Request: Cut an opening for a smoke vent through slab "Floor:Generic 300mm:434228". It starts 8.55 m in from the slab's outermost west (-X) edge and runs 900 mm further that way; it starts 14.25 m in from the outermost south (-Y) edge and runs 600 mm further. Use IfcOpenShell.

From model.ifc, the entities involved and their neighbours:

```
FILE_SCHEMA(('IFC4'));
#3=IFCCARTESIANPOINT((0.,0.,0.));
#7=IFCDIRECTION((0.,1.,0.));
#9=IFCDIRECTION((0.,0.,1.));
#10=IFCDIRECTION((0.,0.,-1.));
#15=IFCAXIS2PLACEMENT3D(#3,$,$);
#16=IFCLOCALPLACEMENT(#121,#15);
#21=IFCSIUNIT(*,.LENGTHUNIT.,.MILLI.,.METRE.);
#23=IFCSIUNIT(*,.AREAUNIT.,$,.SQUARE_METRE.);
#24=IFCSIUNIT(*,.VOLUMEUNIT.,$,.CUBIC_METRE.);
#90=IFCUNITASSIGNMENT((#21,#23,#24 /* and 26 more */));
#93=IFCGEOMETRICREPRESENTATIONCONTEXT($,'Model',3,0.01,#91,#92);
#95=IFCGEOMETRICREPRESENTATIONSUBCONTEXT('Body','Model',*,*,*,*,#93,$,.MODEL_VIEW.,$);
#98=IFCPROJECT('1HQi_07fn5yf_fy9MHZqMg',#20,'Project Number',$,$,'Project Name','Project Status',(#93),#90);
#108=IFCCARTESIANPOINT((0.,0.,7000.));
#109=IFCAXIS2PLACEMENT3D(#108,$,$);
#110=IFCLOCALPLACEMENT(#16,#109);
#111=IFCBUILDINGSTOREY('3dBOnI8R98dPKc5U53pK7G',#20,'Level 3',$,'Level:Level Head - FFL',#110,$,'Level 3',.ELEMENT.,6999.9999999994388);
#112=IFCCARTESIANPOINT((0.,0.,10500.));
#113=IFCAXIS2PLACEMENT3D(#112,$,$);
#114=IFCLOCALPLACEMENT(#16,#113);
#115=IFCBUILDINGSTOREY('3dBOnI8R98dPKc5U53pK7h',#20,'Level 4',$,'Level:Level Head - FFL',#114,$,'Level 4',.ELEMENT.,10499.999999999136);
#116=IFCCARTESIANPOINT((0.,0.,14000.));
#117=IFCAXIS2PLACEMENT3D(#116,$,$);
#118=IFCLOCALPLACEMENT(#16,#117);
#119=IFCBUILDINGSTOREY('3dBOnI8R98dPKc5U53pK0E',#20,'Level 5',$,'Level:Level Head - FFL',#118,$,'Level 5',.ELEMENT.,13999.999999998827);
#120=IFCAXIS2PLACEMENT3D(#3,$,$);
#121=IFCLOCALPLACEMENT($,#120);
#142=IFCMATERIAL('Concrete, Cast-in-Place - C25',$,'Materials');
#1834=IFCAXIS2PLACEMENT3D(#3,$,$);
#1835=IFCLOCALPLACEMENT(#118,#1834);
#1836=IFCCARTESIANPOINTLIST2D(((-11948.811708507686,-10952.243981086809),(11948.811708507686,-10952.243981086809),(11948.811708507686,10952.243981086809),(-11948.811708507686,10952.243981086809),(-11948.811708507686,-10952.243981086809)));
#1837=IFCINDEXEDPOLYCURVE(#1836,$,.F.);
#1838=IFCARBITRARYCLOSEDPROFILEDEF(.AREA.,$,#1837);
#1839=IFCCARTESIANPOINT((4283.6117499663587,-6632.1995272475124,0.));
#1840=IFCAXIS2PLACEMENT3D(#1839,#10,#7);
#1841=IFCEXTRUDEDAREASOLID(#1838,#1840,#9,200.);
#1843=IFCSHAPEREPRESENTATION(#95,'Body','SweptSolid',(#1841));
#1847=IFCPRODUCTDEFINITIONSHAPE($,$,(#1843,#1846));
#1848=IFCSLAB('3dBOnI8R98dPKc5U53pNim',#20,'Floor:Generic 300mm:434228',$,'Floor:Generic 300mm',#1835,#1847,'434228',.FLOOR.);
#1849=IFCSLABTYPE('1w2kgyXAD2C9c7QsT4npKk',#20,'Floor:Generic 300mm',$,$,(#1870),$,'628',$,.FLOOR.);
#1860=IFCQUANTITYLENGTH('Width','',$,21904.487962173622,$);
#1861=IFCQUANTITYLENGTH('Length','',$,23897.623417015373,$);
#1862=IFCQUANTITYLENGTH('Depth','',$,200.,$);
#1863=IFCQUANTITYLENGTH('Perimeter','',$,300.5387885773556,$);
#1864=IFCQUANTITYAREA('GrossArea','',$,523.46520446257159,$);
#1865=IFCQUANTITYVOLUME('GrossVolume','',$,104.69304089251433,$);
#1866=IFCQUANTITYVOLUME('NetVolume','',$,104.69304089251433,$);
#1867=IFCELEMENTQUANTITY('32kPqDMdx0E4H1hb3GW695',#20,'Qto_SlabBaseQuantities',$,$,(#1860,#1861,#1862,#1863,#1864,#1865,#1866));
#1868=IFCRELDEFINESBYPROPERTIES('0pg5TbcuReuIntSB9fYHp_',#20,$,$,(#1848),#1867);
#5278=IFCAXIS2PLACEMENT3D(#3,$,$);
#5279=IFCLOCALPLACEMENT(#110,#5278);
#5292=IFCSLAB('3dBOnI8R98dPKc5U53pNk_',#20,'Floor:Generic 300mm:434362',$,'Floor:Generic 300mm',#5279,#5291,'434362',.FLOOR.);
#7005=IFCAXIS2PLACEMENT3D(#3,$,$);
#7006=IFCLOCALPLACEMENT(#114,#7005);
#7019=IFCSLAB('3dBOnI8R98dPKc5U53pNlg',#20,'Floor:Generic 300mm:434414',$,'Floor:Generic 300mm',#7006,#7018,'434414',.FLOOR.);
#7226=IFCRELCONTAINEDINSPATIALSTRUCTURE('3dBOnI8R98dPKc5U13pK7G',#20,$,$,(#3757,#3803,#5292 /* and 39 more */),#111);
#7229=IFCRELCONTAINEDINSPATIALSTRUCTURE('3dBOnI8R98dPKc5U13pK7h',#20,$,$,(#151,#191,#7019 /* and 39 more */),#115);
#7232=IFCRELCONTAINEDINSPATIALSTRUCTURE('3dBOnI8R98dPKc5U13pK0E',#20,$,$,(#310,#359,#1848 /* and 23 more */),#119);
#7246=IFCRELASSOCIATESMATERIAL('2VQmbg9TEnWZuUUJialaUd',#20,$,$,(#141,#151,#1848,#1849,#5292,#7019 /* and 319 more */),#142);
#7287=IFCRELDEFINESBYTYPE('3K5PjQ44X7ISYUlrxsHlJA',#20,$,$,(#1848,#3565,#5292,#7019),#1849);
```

```python
import numpy as np
import ifcopenshell
import ifcopenshell.api.feature
import ifcopenshell.api.geometry
import ifcopenshell.api.pset
import ifcopenshell.api.root
import ifcopenshell.geom
import ifcopenshell.util.element
import ifcopenshell.util.placement
import ifcopenshell.util.representation
import ifcopenshell.util.shape
import ifcopenshell.util.unit

model = ifcopenshell.open("model.ifc")
unit_scale = ifcopenshell.util.unit.calculate_unit_scale(model)
volume_scale = ifcopenshell.util.unit.calculate_unit_scale(model, "VOLUMEUNIT")
settings = ifcopenshell.geom.settings()


def volume(element):
    """Net volume in cubic metres, openings subtracted."""
    shape = ifcopenshell.geom.create_shape(settings, element)
    return ifcopenshell.util.shape.get_volume(shape.geometry)


slab = model.by_guid("3dBOnI8R98dPKc5U53pNim")
before = volume(slab)

# Extent in the slab's own axes, in metres. The edges named are its -X and -Y sides.
slab_shape = ifcopenshell.geom.create_shape(settings, slab)
vertices = ifcopenshell.util.shape.get_vertices(slab_shape.geometry)
x_min, y_min, bottom = vertices.min(axis=0)
top = vertices[:, 2].max()

opening = ifcopenshell.api.root.create_entity(model, ifc_class="IfcOpeningElement", name="Smoke vent opening", predefined_type="OPENING")
context = ifcopenshell.util.representation.get_context(model, "Model", "Body", "MODEL_VIEW")
width, depth = 0.9, 0.6
outline = [(0.0, 0.0), (width, 0.0), (width, depth), (0.0, depth), (0.0, 0.0)]
# Overshoot both faces by 50 mm so the cut is clean.
shape = ifcopenshell.api.geometry.add_slab_representation(
    model, context=context, depth=top - bottom + 0.1, polyline=outline
)
ifcopenshell.api.geometry.assign_representation(model, product=opening, representation=shape)

matrix = ifcopenshell.util.placement.get_local_placement(slab.ObjectPlacement)
matrix[:, 3] = matrix @ np.append(np.array([x_min + 8.55, y_min + 14.25, bottom - 0.05]) / unit_scale, 1.0)
ifcopenshell.api.geometry.edit_object_placement(model, product=opening, matrix=matrix, is_si=False)
ifcopenshell.api.feature.add_feature(model, feature=opening, element=slab)

after = volume(slab)

# Update the slab's stored quantities.
qto = model.by_id(ifcopenshell.util.element.get_pset(slab, "Qto_SlabBaseQuantities", should_inherit=False)["id"])
ifcopenshell.api.pset.edit_qto(model, qto=qto, properties={"NetVolume": after / volume_scale})

print(f"slab volume {before:.3f} -> {after:.3f} m3")

model.write("model_v2.ifc")
```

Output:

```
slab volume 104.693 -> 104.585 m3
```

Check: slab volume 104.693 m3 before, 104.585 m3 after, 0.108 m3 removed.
